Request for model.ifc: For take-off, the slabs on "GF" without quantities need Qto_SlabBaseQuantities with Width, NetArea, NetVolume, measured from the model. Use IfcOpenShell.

First a look at what the model holds.

```python
import ifcopenshell
import ifcopenshell.util.element
import ifcopenshell.util.unit

model = ifcopenshell.open("model.ifc")
print(model.schema)
for unit_type in ("LENGTHUNIT", "AREAUNIT", "VOLUMEUNIT"):
    print(unit_type, ifcopenshell.util.unit.calculate_unit_scale(model, unit_type))
storey = next(s for s in model.by_type("IfcBuildingStorey") if s.Name == "GF")
slabs = [e for e in ifcopenshell.util.element.get_decomposition(storey) if e.is_a("IfcSlab")]
for e in sorted(slabs, key=lambda e: e.id()):
    print(e.id(), e.is_a(), e.Name, list(ifcopenshell.util.element.get_psets(e, qtos_only=True)), sep=" | ")
```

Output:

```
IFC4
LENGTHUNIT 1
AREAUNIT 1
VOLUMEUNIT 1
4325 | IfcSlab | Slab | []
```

```python
import ifcopenshell
import ifcopenshell.api.pset
import ifcopenshell.geom
import ifcopenshell.util.element
import ifcopenshell.util.shape
import ifcopenshell.util.unit

model = ifcopenshell.open("model.ifc")
unit_scale = ifcopenshell.util.unit.calculate_unit_scale(model)
area_scale = ifcopenshell.util.unit.calculate_unit_scale(model, "AREAUNIT")
volume_scale = ifcopenshell.util.unit.calculate_unit_scale(model, "VOLUMEUNIT")
settings = ifcopenshell.geom.settings()

storey = next(s for s in model.by_type("IfcBuildingStorey") if s.Name == "GF")
slabs = [e for e in ifcopenshell.util.element.get_decomposition(storey) if e.is_a("IfcSlab")]

for e in sorted(slabs, key=lambda e: e.id()):
    if ifcopenshell.util.element.get_psets(e, qtos_only=True, should_inherit=False):
        continue
    # Geometry comes back in metres, in the element's own axes.
    shape = ifcopenshell.geom.create_shape(settings, e)
    values = {
        "Width": ifcopenshell.util.shape.get_z(shape.geometry) / unit_scale,
        "NetArea": ifcopenshell.util.shape.get_footprint_area(shape.geometry) / area_scale,
        "NetVolume": ifcopenshell.util.shape.get_volume(shape.geometry) / volume_scale,
    }
    qto = ifcopenshell.api.pset.add_qto(model, product=e, name="Qto_SlabBaseQuantities")
    ifcopenshell.api.pset.edit_qto(model, qto=qto, properties=values)
    print(e.id(), {k: round(v, 3) for k, v in values.items()})

model.write("model_edited.ifc")
```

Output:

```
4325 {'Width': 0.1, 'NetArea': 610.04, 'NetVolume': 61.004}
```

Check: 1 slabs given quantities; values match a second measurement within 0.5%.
